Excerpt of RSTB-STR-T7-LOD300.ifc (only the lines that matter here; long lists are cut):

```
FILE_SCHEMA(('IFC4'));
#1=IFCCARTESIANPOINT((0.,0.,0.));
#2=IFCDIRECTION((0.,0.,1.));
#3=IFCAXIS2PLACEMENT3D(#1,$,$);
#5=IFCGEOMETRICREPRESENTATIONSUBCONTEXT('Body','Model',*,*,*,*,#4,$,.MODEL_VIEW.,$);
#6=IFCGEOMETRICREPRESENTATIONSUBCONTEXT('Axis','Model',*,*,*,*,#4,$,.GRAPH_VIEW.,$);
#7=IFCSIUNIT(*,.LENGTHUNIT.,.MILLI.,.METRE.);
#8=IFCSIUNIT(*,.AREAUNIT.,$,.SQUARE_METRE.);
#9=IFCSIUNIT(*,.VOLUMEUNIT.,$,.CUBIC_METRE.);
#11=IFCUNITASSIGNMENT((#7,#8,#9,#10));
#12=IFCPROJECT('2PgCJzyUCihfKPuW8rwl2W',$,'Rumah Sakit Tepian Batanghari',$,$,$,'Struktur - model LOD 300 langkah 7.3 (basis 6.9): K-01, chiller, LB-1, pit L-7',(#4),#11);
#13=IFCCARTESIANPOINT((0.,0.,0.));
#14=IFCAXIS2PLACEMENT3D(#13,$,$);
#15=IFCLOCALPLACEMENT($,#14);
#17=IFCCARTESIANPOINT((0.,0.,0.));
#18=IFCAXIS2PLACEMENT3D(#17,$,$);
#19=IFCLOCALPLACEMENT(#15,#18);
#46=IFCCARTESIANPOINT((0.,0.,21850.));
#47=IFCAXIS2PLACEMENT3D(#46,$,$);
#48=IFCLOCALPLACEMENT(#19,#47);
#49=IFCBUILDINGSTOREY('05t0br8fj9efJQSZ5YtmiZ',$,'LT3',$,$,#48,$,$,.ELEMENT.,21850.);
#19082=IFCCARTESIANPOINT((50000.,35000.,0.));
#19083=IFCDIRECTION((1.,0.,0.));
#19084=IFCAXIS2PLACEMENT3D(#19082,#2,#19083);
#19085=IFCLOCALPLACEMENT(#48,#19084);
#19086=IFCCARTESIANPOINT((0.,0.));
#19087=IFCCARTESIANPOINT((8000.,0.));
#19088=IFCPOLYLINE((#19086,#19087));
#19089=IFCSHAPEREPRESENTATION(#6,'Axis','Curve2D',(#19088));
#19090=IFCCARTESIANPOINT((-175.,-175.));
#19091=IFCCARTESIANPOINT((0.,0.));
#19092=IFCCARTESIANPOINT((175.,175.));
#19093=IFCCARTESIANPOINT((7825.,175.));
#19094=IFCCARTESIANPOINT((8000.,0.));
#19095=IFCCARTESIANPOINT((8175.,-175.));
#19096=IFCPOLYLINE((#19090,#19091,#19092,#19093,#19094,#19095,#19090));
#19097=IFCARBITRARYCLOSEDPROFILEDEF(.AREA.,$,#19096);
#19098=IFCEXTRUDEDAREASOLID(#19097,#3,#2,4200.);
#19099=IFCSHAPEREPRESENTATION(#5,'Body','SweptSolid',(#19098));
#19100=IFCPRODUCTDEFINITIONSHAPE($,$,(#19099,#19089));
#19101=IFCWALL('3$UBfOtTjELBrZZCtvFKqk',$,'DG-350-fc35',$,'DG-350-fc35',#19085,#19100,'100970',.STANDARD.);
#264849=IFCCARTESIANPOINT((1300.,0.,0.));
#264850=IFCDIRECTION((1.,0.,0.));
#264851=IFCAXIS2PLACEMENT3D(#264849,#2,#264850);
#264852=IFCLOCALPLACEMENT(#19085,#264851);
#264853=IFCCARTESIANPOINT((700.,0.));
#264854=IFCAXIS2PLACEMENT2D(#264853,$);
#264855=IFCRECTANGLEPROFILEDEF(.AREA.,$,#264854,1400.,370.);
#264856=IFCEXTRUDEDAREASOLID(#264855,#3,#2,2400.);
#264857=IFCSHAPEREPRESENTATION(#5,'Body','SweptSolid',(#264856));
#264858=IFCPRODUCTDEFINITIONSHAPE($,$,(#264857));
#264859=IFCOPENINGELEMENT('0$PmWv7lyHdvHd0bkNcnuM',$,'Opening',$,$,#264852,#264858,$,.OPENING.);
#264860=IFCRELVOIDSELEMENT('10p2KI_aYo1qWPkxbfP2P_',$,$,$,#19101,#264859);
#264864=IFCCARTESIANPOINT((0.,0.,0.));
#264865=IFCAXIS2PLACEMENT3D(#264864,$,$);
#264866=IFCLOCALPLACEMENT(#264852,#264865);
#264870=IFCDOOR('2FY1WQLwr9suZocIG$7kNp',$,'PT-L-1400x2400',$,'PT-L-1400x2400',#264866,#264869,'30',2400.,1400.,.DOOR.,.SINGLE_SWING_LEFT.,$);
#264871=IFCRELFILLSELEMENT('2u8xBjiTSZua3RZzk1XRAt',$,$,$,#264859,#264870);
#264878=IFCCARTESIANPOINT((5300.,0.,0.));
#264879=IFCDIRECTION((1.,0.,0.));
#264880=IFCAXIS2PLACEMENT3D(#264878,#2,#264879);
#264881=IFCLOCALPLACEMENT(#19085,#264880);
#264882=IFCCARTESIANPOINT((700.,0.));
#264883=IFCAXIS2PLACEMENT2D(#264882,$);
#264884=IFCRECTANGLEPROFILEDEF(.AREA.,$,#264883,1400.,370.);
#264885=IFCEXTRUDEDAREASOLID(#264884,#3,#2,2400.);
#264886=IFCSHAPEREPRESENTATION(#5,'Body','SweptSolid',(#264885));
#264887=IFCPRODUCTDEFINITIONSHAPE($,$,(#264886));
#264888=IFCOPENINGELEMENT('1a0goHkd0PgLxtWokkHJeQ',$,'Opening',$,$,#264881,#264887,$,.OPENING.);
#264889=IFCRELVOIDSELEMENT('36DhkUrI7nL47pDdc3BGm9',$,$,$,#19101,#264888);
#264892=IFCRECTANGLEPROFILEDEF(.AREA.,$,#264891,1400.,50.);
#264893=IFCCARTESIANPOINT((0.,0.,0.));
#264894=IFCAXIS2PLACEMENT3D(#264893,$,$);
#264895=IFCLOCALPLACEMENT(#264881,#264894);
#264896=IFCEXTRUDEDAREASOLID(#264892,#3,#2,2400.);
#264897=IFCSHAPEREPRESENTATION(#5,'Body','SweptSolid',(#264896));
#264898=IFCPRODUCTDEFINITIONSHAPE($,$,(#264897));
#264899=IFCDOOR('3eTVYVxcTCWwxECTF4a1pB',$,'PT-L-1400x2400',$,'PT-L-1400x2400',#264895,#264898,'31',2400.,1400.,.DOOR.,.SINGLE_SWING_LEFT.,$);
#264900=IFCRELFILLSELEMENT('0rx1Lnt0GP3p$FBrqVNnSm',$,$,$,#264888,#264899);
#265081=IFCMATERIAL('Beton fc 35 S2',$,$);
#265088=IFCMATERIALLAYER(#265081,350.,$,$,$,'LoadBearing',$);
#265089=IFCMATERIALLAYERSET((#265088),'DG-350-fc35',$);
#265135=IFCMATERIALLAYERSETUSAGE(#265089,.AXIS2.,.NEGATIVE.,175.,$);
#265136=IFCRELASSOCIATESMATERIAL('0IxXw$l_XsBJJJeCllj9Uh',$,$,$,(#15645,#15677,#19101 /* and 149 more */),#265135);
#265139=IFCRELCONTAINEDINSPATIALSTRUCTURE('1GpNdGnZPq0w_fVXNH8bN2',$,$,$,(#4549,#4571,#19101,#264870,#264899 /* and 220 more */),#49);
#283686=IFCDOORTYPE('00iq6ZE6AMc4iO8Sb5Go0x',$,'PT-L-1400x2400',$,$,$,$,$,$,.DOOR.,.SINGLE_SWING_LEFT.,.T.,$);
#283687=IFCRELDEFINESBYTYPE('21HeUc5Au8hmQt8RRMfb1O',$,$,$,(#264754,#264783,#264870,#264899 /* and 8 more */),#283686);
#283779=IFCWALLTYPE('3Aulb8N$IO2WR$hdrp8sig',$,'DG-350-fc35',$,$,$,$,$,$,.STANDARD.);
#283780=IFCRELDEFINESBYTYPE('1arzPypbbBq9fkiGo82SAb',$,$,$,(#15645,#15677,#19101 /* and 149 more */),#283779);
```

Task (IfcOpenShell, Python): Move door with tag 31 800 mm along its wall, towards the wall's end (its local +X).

```python
import ifcopenshell
import ifcopenshell.api.geometry
import ifcopenshell.util.placement
import ifcopenshell.util.unit

model = ifcopenshell.open("RSTB-STR-T7-LOD300.ifc")
unit_scale = ifcopenshell.util.unit.calculate_unit_scale(model)

door = model.by_id(264899)
opening = door.FillsVoids[0].RelatingOpeningElement
wall = opening.VoidsElements[0].RelatingBuildingElement

wall_matrix = ifcopenshell.util.placement.get_local_placement(wall.ObjectPlacement)
shift = wall_matrix[:3, 0] * 0.8 / unit_scale
before = ifcopenshell.util.placement.get_local_placement(door.ObjectPlacement)[:3, 3].copy()

# The door is placed relative to its opening, so it follows when the opening moves.
matrix = ifcopenshell.util.placement.get_local_placement(opening.ObjectPlacement)
matrix[:3, 3] += shift
ifcopenshell.api.geometry.edit_object_placement(
    model, product=opening, matrix=matrix, is_si=False, should_transform_children=True
)

after = ifcopenshell.util.placement.get_local_placement(door.ObjectPlacement)[:3, 3]
print("door moved by", (after - before).round(3) + 0.0)

model.write("RSTB-STR-T7-LOD300_rev.ifc")
```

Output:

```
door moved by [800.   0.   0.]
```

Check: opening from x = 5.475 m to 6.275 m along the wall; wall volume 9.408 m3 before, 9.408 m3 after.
